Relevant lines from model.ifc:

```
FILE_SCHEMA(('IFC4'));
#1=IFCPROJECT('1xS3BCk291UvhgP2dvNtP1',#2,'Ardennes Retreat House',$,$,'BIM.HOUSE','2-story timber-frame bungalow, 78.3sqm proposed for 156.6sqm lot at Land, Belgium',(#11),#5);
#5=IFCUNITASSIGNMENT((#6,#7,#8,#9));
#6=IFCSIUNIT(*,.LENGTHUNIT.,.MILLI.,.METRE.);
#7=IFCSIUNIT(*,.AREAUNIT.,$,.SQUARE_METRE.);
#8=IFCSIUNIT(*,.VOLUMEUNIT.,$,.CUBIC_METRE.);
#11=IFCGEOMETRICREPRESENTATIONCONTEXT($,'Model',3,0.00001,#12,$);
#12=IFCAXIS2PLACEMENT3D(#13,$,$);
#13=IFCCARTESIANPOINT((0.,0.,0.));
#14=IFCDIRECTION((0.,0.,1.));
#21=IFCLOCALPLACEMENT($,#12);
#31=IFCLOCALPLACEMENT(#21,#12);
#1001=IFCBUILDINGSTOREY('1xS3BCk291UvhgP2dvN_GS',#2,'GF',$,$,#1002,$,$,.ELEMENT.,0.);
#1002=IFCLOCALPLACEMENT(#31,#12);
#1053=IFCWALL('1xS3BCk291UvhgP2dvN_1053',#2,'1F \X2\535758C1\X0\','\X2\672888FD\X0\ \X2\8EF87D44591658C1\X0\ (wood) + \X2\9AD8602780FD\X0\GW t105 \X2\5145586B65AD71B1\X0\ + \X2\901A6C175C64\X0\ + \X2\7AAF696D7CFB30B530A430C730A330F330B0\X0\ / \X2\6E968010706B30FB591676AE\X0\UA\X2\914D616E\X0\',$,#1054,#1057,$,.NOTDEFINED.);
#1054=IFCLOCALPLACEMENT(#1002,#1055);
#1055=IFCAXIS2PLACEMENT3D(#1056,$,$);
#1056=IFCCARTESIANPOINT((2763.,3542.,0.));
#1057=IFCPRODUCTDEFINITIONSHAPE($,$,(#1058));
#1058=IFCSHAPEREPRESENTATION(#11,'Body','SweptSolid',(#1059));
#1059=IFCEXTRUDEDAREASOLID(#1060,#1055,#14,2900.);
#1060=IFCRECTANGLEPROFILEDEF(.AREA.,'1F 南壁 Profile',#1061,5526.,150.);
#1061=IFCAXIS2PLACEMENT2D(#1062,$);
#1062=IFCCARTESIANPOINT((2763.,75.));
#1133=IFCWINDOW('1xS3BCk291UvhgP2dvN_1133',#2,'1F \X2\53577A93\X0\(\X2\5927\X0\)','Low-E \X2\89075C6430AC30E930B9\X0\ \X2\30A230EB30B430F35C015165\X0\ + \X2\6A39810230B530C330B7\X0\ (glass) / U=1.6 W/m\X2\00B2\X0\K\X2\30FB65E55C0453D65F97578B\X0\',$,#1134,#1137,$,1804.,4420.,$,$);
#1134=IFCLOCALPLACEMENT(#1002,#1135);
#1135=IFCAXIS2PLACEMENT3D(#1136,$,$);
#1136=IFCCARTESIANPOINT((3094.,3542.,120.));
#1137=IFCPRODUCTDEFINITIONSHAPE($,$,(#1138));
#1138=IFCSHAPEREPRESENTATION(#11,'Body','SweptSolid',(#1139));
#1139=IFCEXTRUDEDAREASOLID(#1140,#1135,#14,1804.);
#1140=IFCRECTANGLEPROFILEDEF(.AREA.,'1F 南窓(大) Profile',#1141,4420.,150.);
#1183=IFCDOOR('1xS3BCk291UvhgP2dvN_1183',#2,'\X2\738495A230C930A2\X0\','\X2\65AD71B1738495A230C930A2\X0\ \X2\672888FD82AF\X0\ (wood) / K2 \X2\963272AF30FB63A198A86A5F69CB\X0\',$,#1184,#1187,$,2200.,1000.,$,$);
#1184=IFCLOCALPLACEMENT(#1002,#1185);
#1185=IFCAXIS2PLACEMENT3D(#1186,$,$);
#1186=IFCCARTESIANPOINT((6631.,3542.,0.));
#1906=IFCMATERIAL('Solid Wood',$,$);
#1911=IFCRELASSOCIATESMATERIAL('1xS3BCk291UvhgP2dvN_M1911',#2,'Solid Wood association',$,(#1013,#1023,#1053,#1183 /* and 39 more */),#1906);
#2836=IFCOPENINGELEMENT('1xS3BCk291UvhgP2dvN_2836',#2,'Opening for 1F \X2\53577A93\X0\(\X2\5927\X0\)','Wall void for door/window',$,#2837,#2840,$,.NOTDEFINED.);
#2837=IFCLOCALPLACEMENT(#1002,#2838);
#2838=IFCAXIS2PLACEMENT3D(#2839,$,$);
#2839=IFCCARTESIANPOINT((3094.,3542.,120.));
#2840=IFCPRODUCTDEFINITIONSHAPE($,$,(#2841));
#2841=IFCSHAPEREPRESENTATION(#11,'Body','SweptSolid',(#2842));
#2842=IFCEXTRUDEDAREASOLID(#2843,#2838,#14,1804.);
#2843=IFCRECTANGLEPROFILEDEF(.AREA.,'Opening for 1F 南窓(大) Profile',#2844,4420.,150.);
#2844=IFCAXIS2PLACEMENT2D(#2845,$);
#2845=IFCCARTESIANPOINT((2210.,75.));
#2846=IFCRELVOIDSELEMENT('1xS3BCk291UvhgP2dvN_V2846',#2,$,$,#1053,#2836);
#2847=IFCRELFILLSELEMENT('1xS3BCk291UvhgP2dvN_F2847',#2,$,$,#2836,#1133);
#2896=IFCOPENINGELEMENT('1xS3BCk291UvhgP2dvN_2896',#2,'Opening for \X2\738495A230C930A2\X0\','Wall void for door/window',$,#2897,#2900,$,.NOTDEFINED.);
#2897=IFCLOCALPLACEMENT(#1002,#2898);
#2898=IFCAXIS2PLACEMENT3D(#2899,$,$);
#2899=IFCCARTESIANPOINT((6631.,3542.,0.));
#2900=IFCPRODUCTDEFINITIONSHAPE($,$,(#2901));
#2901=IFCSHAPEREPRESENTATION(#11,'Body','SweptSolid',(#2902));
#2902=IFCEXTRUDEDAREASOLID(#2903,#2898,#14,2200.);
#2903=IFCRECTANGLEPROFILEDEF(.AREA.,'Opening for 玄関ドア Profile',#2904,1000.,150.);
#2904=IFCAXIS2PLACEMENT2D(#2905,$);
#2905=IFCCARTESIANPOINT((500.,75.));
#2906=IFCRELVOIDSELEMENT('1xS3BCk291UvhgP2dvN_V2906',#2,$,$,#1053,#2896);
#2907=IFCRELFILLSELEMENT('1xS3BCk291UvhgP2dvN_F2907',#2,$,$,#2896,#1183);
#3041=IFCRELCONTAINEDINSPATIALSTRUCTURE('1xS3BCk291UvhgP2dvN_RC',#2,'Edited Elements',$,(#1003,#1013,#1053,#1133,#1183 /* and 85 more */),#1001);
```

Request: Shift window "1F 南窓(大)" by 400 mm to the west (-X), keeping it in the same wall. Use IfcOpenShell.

```python
import ifcopenshell
import ifcopenshell.api.geometry
import ifcopenshell.util.placement

model = ifcopenshell.open("model.ifc")

window = model.by_guid("1xS3BCk291UvhgP2dvN_1133")
opening = window.FillsVoids[0].RelatingOpeningElement
wall = opening.VoidsElements[0].RelatingBuildingElement

wall_matrix = ifcopenshell.util.placement.get_local_placement(wall.ObjectPlacement)
shift = wall_matrix[:3, 0] * -400.0
before = ifcopenshell.util.placement.get_local_placement(window.ObjectPlacement)[:3, 3].copy()

# The window is not placed relative to its opening, so move both.
for product in (opening, window):
    matrix = ifcopenshell.util.placement.get_local_placement(product.ObjectPlacement)
    matrix[:3, 3] += shift
    ifcopenshell.api.geometry.edit_object_placement(model, product=product, matrix=matrix, is_si=False)

after = ifcopenshell.util.placement.get_local_placement(window.ObjectPlacement)[:3, 3]
print("window moved by", (after - before).round(3) + 0.0)

model.write("model-out.ifc")
```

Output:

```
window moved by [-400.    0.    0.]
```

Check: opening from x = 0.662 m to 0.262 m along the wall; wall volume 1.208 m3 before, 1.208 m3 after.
